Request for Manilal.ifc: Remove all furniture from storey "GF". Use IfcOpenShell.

First a look at what the model holds.

```python
import ifcopenshell
import ifcopenshell.util.element

model = ifcopenshell.open("Manilal.ifc")
print(model.schema)
storey = next(s for s in model.by_type("IfcBuildingStorey") if s.Name == "GF")
furniture = [e for e in ifcopenshell.util.element.get_decomposition(storey) if e.is_a("IfcFurnishingElement")]
seen = {}
for e in furniture:
    element_type = ifcopenshell.util.element.get_type(e)
    name = element_type.Name if element_type not in (None, e) else None
    seen[name] = seen.get(name, 0) + 1
for name, count in sorted(seen.items(), key=str):
    print(count, "x", name)
```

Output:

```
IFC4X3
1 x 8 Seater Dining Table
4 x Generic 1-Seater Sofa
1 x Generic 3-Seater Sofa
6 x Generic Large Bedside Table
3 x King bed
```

```python
import ifcopenshell
import ifcopenshell.api.root
import ifcopenshell.util.element

model = ifcopenshell.open("Manilal.ifc")

storey = next(s for s in model.by_type("IfcBuildingStorey") if s.Name == "GF")
furniture = [e for e in ifcopenshell.util.element.get_decomposition(storey) if e.is_a("IfcFurnishingElement")]

for e in furniture:
    ifcopenshell.api.root.remove_product(model, product=e)
print(len(furniture), "removed")

model.write("Manilal-out.ifc")
```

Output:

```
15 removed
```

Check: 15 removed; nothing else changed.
